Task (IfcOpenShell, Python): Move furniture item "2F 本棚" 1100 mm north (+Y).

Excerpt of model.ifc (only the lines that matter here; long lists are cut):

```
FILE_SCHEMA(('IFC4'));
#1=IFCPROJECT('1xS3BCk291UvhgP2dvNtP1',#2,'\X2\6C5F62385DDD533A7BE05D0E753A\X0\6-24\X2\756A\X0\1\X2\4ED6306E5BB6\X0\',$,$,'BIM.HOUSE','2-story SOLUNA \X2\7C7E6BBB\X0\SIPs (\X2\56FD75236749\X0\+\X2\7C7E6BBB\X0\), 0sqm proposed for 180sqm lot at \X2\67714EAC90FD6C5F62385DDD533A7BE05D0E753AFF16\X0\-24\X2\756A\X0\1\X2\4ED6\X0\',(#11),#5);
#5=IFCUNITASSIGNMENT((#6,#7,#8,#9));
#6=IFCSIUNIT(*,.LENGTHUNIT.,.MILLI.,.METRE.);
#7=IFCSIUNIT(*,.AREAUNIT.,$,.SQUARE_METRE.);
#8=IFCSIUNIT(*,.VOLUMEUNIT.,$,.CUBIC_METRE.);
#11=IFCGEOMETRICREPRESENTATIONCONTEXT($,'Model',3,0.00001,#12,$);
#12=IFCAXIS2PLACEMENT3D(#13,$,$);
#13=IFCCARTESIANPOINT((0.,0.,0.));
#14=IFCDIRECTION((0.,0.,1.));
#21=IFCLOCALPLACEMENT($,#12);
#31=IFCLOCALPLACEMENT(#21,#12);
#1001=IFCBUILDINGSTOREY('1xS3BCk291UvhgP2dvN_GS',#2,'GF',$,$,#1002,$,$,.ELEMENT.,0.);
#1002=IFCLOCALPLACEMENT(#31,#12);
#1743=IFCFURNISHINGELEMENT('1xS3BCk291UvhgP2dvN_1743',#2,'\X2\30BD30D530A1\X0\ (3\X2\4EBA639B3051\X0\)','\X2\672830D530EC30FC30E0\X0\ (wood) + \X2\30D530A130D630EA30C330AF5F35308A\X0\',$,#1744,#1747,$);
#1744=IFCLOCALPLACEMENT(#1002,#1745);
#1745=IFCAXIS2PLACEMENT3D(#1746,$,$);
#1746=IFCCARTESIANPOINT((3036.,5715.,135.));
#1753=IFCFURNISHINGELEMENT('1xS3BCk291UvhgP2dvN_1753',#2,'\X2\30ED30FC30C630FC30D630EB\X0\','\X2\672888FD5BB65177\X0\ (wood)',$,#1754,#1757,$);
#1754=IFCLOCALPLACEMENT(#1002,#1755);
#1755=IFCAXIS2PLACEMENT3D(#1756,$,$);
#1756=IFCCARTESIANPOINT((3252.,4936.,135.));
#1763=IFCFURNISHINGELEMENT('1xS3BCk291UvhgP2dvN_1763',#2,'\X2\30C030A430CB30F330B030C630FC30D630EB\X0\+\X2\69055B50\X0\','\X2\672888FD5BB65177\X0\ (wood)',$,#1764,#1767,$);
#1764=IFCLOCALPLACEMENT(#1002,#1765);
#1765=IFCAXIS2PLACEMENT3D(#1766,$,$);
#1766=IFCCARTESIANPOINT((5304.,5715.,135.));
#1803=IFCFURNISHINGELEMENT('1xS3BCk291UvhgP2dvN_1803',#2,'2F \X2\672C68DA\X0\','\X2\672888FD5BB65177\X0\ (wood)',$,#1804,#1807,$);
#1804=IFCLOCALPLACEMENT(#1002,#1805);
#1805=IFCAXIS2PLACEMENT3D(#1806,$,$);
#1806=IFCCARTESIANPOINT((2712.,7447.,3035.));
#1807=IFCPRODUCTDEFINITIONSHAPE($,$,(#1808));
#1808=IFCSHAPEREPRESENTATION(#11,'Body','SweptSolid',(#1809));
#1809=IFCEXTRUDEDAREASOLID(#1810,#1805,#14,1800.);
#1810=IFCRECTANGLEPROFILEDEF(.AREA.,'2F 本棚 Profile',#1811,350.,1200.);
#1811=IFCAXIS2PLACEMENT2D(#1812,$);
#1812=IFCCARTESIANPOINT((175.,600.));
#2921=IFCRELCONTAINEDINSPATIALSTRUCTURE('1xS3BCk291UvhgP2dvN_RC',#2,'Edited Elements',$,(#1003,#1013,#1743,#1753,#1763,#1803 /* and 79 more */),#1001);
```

```python
import ifcopenshell
import ifcopenshell.api.geometry
import ifcopenshell.util.placement

model = ifcopenshell.open("model.ifc")

item = model.by_id(1803)
matrix = ifcopenshell.util.placement.get_local_placement(item.ObjectPlacement)
matrix[1, 3] += 1100.0
ifcopenshell.api.geometry.edit_object_placement(model, product=item, matrix=matrix, is_si=False)

print(ifcopenshell.util.placement.get_local_placement(item.ObjectPlacement).round(3) + 0.0)

model.write("model_rev.ifc")
```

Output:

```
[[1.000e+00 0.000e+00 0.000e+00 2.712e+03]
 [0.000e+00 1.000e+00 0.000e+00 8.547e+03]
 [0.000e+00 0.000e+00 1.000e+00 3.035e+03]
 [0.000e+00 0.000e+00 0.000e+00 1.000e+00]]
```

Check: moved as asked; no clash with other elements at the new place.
